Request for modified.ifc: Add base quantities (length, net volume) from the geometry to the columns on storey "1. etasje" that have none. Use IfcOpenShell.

First a look at what the model holds.

```python
import ifcopenshell
import ifcopenshell.util.element
import ifcopenshell.util.unit

model = ifcopenshell.open("modified.ifc")
print(model.schema)
for unit_type in ("LENGTHUNIT", "AREAUNIT", "VOLUMEUNIT"):
    print(unit_type, ifcopenshell.util.unit.calculate_unit_scale(model, unit_type))
storey = next(s for s in model.by_type("IfcBuildingStorey") if s.Name == "1. etasje")
columns = [e for e in ifcopenshell.util.element.get_decomposition(storey) if e.is_a("IfcColumn")]
for e in sorted(columns, key=lambda e: e.id()):
    print(e.id(), e.is_a(), e.Name, list(ifcopenshell.util.element.get_psets(e, qtos_only=True)), sep=" | ")
```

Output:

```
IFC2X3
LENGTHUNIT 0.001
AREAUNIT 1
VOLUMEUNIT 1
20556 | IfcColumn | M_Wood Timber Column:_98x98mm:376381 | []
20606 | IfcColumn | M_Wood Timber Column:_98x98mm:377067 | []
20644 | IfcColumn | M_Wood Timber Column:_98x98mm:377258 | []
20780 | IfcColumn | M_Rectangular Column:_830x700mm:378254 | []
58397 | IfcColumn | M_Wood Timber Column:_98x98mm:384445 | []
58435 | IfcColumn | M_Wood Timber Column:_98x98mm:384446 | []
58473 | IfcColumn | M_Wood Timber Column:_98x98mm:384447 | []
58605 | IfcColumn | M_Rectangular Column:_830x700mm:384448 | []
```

```python
import ifcopenshell
import ifcopenshell.api.pset
import ifcopenshell.geom
import ifcopenshell.util.element
import ifcopenshell.util.shape
import ifcopenshell.util.unit

model = ifcopenshell.open("modified.ifc")
unit_scale = ifcopenshell.util.unit.calculate_unit_scale(model)
volume_scale = ifcopenshell.util.unit.calculate_unit_scale(model, "VOLUMEUNIT")
settings = ifcopenshell.geom.settings()

storey = next(s for s in model.by_type("IfcBuildingStorey") if s.Name == "1. etasje")
columns = [e for e in ifcopenshell.util.element.get_decomposition(storey) if e.is_a("IfcColumn")]

for e in sorted(columns, key=lambda e: e.id()):
    if ifcopenshell.util.element.get_psets(e, qtos_only=True, should_inherit=False):
        continue
    # Geometry comes back in metres, in the element's own axes.
    shape = ifcopenshell.geom.create_shape(settings, e)
    values = {
        "Length": ifcopenshell.util.shape.get_z(shape.geometry) / unit_scale,
        "NetVolume": ifcopenshell.util.shape.get_volume(shape.geometry) / volume_scale,
    }
    qto = ifcopenshell.api.pset.add_qto(model, product=e, name="BaseQuantities")
    ifcopenshell.api.pset.edit_qto(model, qto=qto, properties=values)
    print(e.id(), {k: round(v, 3) for k, v in values.items()})

model.write("modified_v2.ifc")
```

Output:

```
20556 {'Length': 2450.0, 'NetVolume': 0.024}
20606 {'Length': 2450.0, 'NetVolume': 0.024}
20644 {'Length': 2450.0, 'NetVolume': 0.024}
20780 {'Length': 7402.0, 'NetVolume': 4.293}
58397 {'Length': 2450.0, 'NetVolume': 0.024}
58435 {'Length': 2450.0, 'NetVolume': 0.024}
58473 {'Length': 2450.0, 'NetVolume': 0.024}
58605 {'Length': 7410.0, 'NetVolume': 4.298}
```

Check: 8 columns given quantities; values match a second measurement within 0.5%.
